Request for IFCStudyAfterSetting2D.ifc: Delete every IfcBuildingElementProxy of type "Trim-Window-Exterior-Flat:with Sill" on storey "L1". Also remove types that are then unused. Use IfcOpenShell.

First a look at what the model holds.

```python
import ifcopenshell
import ifcopenshell.util.element

model = ifcopenshell.open("IFCStudyAfterSetting2D.ifc")
print(model.schema)
storey = next(s for s in model.by_type("IfcBuildingStorey") if s.Name == "L1")
proxies = [e for e in ifcopenshell.util.element.get_decomposition(storey) if e.is_a("IfcBuildingElementProxy")]
seen = {}
for e in proxies:
    element_type = ifcopenshell.util.element.get_type(e)
    name = element_type.Name if element_type not in (None, e) else None
    seen[name] = seen.get(name, 0) + 1
for name, count in sorted(seen.items(), key=str):
    print(count, "x", name)
```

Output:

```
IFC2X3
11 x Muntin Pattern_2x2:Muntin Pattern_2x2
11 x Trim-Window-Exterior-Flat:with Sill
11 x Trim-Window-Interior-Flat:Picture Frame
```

```python
import ifcopenshell
import ifcopenshell.api.root
import ifcopenshell.util.element

model = ifcopenshell.open("IFCStudyAfterSetting2D.ifc")

storey = next(s for s in model.by_type("IfcBuildingStorey") if s.Name == "L1")
proxies = [e for e in ifcopenshell.util.element.get_decomposition(storey) if e.is_a("IfcBuildingElementProxy")]
targets = [e for e in proxies if (t := ifcopenshell.util.element.get_type(e)) not in (None, e) and t.Name == "Trim-Window-Exterior-Flat:with Sill"]
types = {ifcopenshell.util.element.get_type(e) for e in targets} - {None, *targets}

for e in targets:
    ifcopenshell.api.root.remove_product(model, product=e)
print(len(targets), "removed")

unused = [t for t in types if not ifcopenshell.util.element.get_types(t)]
for t in unused:
    ifcopenshell.api.root.remove_product(model, product=t)
print(len(unused), "unused types removed")

model.write("IFCStudyAfterSetting2D_v2.ifc")
```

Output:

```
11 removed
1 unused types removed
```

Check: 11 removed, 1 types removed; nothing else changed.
